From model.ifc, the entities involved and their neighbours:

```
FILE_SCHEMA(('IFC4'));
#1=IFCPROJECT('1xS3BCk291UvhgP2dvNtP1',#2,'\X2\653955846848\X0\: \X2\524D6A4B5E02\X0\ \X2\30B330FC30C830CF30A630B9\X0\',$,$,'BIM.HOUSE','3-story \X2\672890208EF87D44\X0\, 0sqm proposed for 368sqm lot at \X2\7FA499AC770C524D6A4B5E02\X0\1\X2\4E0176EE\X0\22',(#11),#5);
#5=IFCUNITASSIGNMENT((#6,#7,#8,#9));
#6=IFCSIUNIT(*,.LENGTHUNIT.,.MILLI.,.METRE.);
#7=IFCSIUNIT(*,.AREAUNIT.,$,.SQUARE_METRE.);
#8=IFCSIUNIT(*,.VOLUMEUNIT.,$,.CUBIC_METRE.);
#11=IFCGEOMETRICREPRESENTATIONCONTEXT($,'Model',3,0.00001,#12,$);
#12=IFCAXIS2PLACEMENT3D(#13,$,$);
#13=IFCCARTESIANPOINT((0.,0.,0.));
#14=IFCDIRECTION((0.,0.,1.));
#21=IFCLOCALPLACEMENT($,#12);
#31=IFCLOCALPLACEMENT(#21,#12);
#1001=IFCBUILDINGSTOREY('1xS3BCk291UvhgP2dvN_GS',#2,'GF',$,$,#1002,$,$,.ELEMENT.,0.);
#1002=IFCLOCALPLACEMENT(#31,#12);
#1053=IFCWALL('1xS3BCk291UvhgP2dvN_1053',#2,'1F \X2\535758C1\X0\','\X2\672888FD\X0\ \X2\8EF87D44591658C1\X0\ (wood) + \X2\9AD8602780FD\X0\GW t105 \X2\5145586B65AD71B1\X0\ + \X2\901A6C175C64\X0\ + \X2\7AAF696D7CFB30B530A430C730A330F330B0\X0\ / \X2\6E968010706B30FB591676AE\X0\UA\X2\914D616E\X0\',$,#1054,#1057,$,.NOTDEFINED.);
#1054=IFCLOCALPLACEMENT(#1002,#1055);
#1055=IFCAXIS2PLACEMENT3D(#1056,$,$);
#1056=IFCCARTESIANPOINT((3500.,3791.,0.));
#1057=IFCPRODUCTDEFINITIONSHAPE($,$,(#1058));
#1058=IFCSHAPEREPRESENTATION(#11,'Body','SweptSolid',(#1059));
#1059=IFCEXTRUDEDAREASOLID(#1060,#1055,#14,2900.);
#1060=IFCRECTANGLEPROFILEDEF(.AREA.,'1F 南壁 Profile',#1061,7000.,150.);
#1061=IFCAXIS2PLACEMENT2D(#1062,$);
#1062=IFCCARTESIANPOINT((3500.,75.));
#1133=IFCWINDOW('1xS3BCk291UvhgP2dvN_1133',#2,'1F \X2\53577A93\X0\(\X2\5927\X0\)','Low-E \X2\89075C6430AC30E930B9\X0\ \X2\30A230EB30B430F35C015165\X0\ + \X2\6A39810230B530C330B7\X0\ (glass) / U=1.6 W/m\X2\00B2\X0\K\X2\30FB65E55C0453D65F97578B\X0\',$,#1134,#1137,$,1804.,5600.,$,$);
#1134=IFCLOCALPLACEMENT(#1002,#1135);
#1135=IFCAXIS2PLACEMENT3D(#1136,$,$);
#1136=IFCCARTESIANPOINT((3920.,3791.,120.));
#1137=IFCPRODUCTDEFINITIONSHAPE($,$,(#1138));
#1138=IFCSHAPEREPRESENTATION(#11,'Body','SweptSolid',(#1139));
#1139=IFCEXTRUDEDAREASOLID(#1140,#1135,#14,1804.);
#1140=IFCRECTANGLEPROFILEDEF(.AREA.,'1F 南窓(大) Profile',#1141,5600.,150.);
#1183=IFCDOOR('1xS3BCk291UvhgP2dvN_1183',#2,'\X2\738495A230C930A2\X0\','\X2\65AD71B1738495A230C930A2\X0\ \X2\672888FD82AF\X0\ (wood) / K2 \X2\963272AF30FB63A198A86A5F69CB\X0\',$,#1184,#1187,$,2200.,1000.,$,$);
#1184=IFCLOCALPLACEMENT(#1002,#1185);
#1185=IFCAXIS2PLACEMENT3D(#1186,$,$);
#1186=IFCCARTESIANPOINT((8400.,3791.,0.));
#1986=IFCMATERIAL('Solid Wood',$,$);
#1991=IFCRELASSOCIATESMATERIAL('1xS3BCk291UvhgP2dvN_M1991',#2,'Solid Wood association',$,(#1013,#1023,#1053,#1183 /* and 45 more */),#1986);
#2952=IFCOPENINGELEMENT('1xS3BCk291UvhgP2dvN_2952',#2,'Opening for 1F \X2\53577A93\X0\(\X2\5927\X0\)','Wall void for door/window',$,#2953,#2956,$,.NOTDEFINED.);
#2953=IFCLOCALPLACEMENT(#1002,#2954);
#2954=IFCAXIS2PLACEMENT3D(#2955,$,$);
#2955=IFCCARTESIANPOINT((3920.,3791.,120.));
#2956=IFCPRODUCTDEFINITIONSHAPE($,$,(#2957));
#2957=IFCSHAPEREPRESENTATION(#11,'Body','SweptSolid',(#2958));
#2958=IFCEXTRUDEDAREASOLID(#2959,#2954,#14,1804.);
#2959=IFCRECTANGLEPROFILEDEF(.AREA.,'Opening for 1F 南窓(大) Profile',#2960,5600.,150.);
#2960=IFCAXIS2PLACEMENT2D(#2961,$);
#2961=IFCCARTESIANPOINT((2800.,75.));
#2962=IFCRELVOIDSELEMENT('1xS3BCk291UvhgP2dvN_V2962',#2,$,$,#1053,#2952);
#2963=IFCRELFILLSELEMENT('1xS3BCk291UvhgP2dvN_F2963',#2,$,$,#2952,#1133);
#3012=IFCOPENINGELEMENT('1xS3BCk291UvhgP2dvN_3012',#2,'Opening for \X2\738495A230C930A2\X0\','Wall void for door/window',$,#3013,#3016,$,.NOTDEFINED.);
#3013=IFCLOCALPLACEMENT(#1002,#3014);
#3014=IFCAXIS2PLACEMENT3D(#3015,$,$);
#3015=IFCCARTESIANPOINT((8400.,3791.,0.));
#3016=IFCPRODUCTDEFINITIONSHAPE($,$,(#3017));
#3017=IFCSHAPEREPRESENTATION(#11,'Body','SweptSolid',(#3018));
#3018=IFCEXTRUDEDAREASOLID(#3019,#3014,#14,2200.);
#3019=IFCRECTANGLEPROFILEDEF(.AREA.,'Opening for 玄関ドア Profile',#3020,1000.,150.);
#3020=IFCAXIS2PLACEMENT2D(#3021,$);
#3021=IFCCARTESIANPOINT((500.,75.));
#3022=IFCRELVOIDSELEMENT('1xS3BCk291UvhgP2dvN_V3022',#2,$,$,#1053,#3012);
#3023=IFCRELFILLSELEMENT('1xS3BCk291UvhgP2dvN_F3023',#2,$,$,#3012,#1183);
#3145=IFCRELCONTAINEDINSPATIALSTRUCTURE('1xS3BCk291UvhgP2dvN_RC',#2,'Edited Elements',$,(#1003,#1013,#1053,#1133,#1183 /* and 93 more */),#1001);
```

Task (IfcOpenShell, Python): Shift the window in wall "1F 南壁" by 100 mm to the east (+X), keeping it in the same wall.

```python
import ifcopenshell
import ifcopenshell.api.geometry
import ifcopenshell.util.placement

model = ifcopenshell.open("model.ifc")

window = model.by_guid("1xS3BCk291UvhgP2dvN_1133")
opening = window.FillsVoids[0].RelatingOpeningElement
wall = opening.VoidsElements[0].RelatingBuildingElement

wall_matrix = ifcopenshell.util.placement.get_local_placement(wall.ObjectPlacement)
shift = wall_matrix[:3, 0] * 100.0
before = ifcopenshell.util.placement.get_local_placement(window.ObjectPlacement)[:3, 3].copy()

# The window is not placed relative to its opening, so move both.
for product in (opening, window):
    matrix = ifcopenshell.util.placement.get_local_placement(product.ObjectPlacement)
    matrix[:3, 3] += shift
    ifcopenshell.api.geometry.edit_object_placement(model, product=product, matrix=matrix, is_si=False)

after = ifcopenshell.util.placement.get_local_placement(window.ObjectPlacement)[:3, 3]
print("window moved by", (after - before).round(3) + 0.0)

model.write("model-out.ifc")
```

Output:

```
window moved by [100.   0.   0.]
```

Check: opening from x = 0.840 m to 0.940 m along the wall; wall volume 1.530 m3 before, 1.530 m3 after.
